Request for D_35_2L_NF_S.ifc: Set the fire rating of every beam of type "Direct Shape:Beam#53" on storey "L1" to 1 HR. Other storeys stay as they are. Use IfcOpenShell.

First a look at what the model holds.

```python
import ifcopenshell
import ifcopenshell.util.element

model = ifcopenshell.open("D_35_2L_NF_S.ifc")
print(model.schema)
storey = next(s for s in model.by_type("IfcBuildingStorey") if s.Name == "L1")
beams = [e for e in ifcopenshell.util.element.get_decomposition(storey) if e.is_a("IfcBeam")]
seen = {}
for e in beams:
    element_type = ifcopenshell.util.element.get_type(e)
    key = (element_type.Name if element_type != e and element_type else None, ifcopenshell.util.element.get_pset(e, "Pset_BeamCommon", "FireRating"))
    seen[key] = seen.get(key, 0) + 1
for (name, value), count in sorted(seen.items(), key=str):
    print(count, "x", name, "|", value)
```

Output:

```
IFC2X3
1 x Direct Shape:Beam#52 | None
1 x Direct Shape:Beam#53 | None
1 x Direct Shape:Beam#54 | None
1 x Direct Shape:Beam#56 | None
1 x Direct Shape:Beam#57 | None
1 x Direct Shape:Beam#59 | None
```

```python
import ifcopenshell
import ifcopenshell.api.pset
import ifcopenshell.util.element

model = ifcopenshell.open("D_35_2L_NF_S.ifc")

storey = next(s for s in model.by_type("IfcBuildingStorey") if s.Name == "L1")
beams = [e for e in ifcopenshell.util.element.get_decomposition(storey) if e.is_a("IfcBeam")]

count = 0
for e in beams:
    element_type = ifcopenshell.util.element.get_type(e)
    if element_type in (None, e) or element_type.Name != "Direct Shape:Beam#53":
        continue
    # add_pset returns the element's existing set when there is one.
    pset = ifcopenshell.api.pset.add_pset(model, product=e, name="Pset_BeamCommon")
    ifcopenshell.api.pset.edit_pset(model, pset=pset, properties={"FireRating": "1 HR"})
    count += 1

print(count, "beams updated")

model.write("D_35_2L_NF_S_rev.ifc")
```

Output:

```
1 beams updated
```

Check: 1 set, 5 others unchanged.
